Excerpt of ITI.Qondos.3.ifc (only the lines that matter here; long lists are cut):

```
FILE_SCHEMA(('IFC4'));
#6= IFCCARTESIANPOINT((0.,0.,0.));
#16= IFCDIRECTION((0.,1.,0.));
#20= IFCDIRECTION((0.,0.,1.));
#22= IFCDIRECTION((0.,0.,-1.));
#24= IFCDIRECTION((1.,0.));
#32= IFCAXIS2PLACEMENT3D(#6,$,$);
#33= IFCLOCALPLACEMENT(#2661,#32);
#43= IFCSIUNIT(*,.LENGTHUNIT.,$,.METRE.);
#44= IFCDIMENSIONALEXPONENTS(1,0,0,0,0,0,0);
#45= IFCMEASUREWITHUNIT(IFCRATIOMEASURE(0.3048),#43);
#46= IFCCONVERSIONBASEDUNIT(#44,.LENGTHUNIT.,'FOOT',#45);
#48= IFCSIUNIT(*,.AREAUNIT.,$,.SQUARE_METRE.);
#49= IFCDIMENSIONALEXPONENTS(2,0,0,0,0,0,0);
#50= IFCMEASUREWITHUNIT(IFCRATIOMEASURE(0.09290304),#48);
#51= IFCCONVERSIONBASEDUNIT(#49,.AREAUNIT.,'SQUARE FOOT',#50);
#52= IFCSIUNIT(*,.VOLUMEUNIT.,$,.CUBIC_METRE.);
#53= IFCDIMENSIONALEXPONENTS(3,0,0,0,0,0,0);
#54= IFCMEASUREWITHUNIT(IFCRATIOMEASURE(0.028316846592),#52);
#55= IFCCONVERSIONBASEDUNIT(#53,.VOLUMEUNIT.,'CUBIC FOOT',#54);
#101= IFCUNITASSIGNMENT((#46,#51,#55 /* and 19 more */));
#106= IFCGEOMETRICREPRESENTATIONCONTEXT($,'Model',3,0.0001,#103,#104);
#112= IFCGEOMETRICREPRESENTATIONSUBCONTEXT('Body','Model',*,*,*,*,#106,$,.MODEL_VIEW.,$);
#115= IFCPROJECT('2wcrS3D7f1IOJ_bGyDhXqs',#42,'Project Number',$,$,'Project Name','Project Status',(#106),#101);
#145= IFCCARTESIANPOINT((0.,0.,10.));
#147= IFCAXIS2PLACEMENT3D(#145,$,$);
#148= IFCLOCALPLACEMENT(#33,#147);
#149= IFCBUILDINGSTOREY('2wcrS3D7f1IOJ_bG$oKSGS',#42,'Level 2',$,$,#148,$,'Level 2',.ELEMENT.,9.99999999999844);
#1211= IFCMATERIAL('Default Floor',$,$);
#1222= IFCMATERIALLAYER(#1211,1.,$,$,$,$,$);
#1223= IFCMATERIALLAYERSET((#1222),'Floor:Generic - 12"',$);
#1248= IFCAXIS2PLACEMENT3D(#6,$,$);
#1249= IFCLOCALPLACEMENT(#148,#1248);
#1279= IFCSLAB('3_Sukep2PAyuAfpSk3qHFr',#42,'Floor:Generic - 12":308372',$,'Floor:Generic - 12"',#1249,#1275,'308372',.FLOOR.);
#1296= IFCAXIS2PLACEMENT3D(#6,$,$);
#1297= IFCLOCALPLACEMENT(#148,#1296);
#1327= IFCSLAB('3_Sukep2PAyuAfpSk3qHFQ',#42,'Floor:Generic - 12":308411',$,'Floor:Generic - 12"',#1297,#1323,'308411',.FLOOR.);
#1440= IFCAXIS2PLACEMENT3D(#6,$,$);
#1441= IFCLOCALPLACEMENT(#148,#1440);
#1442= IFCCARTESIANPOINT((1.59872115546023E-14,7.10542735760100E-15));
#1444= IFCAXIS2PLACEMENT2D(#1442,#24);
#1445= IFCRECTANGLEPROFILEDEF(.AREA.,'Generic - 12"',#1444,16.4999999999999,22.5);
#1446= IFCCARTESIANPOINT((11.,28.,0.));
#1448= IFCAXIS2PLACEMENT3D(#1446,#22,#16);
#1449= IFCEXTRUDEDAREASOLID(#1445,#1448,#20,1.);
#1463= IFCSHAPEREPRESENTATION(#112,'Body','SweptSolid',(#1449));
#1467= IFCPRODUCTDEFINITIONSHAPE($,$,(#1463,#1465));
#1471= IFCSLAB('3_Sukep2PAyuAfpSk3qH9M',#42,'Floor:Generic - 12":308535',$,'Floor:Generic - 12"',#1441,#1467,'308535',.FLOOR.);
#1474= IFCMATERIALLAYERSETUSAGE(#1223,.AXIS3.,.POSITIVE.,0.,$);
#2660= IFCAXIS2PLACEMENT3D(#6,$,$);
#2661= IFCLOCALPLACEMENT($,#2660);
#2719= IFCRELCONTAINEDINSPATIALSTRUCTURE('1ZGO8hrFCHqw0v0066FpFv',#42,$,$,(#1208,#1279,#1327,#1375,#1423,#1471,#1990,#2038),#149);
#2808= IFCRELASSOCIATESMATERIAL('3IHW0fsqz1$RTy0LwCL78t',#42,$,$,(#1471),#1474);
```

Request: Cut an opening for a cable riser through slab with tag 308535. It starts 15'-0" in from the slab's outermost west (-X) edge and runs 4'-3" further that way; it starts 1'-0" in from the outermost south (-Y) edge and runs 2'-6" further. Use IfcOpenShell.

```python
import numpy as np
import ifcopenshell
import ifcopenshell.api.feature
import ifcopenshell.api.geometry
import ifcopenshell.api.root
import ifcopenshell.geom
import ifcopenshell.util.placement
import ifcopenshell.util.representation
import ifcopenshell.util.shape
import ifcopenshell.util.unit

model = ifcopenshell.open("ITI.Qondos.3.ifc")
unit_scale = ifcopenshell.util.unit.calculate_unit_scale(model)
settings = ifcopenshell.geom.settings()


def volume(element):
    """Net volume in cubic metres, openings subtracted."""
    shape = ifcopenshell.geom.create_shape(settings, element)
    return ifcopenshell.util.shape.get_volume(shape.geometry)


slab = model.by_guid("3_Sukep2PAyuAfpSk3qH9M")
before = volume(slab)

# Extent in the slab's own axes, in metres. The edges named are its -X and -Y sides.
slab_shape = ifcopenshell.geom.create_shape(settings, slab)
vertices = ifcopenshell.util.shape.get_vertices(slab_shape.geometry)
x_min, y_min, bottom = vertices.min(axis=0)
top = vertices[:, 2].max()

opening = ifcopenshell.api.root.create_entity(model, ifc_class="IfcOpeningElement", name="Cable riser opening", predefined_type="OPENING")
context = ifcopenshell.util.representation.get_context(model, "Model", "Body", "MODEL_VIEW")
width, depth = 1.2954, 0.762
outline = [(0.0, 0.0), (width, 0.0), (width, depth), (0.0, depth), (0.0, 0.0)]
# Overshoot both faces by 50 mm so the cut is clean.
shape = ifcopenshell.api.geometry.add_slab_representation(
    model, context=context, depth=top - bottom + 0.1, polyline=outline
)
ifcopenshell.api.geometry.assign_representation(model, product=opening, representation=shape)

matrix = ifcopenshell.util.placement.get_local_placement(slab.ObjectPlacement)
matrix[:, 3] = matrix @ np.append(np.array([x_min + 4.572, y_min + 0.3048, bottom - 0.05]) / unit_scale, 1.0)
ifcopenshell.api.geometry.edit_object_placement(model, product=opening, matrix=matrix, is_si=False)
ifcopenshell.api.feature.add_feature(model, feature=opening, element=slab)

after = volume(slab)

print(f"slab volume {before:.3f} -> {after:.3f} m3")

model.write("ITI.Qondos.3_rev.ifc")
```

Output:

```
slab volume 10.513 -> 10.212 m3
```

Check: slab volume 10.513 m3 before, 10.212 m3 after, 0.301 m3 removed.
